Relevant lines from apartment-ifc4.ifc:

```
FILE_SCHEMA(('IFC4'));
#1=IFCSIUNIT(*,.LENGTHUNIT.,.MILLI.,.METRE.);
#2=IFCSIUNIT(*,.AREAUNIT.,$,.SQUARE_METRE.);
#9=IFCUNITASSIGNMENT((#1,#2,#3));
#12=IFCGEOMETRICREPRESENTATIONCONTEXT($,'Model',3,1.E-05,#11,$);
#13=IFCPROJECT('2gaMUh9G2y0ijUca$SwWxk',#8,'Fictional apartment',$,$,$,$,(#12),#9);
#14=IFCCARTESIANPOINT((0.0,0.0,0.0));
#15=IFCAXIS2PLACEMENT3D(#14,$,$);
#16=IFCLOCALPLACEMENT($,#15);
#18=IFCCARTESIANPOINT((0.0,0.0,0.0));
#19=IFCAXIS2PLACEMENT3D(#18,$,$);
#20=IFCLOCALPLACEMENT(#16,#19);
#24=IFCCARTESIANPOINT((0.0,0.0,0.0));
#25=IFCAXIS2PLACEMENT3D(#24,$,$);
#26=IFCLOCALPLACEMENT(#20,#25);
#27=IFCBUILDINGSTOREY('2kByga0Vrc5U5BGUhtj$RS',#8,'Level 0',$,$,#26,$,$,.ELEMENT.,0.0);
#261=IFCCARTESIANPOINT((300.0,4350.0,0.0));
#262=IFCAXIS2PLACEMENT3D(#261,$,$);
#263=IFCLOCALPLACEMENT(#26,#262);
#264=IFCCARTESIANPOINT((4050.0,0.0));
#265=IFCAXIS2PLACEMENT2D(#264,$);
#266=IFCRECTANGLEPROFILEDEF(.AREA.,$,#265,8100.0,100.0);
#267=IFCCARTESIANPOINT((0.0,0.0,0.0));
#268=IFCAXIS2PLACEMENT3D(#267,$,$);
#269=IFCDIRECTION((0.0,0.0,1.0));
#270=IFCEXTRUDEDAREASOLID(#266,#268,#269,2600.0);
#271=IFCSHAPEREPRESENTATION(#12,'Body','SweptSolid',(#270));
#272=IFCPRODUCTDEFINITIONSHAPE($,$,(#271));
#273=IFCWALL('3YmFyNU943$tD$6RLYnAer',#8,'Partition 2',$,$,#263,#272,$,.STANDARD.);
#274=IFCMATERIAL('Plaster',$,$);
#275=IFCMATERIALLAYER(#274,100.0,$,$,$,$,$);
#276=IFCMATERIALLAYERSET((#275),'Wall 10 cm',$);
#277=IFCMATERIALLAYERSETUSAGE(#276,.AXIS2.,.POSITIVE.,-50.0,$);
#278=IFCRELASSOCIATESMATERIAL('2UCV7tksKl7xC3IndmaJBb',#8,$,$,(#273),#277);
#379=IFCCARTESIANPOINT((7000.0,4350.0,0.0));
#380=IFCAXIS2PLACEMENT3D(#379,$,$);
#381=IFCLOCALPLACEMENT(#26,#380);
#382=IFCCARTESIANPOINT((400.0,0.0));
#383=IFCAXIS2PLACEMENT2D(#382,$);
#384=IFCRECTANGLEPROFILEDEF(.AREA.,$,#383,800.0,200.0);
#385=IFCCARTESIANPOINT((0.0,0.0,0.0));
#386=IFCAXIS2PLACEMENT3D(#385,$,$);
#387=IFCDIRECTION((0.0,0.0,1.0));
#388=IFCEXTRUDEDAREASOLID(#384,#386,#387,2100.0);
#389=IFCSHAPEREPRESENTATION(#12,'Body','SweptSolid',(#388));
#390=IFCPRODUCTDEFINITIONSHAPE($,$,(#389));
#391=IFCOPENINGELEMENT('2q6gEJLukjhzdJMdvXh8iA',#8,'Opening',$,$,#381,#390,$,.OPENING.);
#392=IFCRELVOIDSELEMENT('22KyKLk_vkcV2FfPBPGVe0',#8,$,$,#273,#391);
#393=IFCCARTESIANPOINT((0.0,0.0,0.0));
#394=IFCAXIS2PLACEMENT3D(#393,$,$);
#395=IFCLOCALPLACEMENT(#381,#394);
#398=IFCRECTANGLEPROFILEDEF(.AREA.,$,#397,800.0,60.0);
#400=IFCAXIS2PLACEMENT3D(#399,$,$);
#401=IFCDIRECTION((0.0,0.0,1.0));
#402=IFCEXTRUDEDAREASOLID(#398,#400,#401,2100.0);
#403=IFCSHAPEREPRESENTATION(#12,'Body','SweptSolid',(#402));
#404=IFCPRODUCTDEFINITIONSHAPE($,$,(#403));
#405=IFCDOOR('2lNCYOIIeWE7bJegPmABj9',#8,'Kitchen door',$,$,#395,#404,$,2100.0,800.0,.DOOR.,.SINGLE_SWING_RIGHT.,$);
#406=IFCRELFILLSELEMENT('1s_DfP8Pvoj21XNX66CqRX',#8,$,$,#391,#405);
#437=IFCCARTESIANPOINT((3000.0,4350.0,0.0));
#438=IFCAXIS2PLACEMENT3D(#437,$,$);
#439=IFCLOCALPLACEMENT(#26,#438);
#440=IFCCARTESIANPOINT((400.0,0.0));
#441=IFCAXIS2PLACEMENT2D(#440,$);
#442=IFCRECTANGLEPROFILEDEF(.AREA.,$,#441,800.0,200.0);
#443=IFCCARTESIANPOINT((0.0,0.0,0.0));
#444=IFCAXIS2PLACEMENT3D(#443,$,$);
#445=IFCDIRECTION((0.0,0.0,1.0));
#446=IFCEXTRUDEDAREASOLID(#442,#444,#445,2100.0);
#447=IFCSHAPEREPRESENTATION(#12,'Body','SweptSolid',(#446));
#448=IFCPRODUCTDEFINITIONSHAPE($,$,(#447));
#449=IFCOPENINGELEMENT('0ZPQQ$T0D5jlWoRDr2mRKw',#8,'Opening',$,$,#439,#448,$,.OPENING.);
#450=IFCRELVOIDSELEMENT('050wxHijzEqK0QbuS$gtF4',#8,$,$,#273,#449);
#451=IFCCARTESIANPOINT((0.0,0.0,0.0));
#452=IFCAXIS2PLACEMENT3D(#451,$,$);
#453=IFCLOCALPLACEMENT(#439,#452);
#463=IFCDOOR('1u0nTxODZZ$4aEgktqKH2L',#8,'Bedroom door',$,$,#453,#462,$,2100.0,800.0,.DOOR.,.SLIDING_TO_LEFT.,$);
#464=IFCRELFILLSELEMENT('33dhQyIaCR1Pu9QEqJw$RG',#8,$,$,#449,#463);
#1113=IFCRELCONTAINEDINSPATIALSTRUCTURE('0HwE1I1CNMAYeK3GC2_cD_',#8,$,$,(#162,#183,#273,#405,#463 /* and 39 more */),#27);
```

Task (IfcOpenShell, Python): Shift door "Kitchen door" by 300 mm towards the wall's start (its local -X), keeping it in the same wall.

```python
import ifcopenshell
import ifcopenshell.api.geometry
import ifcopenshell.util.placement
import ifcopenshell.util.unit

model = ifcopenshell.open("apartment-ifc4.ifc")
unit_scale = ifcopenshell.util.unit.calculate_unit_scale(model)

door = model.by_guid("2lNCYOIIeWE7bJegPmABj9")
opening = door.FillsVoids[0].RelatingOpeningElement
wall = opening.VoidsElements[0].RelatingBuildingElement

wall_matrix = ifcopenshell.util.placement.get_local_placement(wall.ObjectPlacement)
shift = wall_matrix[:3, 0] * -0.3 / unit_scale
before = ifcopenshell.util.placement.get_local_placement(door.ObjectPlacement)[:3, 3].copy()

# The door is placed relative to its opening, so it follows when the opening moves.
matrix = ifcopenshell.util.placement.get_local_placement(opening.ObjectPlacement)
matrix[:3, 3] += shift
ifcopenshell.api.geometry.edit_object_placement(
    model, product=opening, matrix=matrix, is_si=False, should_transform_children=True
)

after = ifcopenshell.util.placement.get_local_placement(door.ObjectPlacement)[:3, 3]
print("door moved by", (after - before).round(3) + 0.0)

model.write("apartment-ifc4_updated.ifc")
```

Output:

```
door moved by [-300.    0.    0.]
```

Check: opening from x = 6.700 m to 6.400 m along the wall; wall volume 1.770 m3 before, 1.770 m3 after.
